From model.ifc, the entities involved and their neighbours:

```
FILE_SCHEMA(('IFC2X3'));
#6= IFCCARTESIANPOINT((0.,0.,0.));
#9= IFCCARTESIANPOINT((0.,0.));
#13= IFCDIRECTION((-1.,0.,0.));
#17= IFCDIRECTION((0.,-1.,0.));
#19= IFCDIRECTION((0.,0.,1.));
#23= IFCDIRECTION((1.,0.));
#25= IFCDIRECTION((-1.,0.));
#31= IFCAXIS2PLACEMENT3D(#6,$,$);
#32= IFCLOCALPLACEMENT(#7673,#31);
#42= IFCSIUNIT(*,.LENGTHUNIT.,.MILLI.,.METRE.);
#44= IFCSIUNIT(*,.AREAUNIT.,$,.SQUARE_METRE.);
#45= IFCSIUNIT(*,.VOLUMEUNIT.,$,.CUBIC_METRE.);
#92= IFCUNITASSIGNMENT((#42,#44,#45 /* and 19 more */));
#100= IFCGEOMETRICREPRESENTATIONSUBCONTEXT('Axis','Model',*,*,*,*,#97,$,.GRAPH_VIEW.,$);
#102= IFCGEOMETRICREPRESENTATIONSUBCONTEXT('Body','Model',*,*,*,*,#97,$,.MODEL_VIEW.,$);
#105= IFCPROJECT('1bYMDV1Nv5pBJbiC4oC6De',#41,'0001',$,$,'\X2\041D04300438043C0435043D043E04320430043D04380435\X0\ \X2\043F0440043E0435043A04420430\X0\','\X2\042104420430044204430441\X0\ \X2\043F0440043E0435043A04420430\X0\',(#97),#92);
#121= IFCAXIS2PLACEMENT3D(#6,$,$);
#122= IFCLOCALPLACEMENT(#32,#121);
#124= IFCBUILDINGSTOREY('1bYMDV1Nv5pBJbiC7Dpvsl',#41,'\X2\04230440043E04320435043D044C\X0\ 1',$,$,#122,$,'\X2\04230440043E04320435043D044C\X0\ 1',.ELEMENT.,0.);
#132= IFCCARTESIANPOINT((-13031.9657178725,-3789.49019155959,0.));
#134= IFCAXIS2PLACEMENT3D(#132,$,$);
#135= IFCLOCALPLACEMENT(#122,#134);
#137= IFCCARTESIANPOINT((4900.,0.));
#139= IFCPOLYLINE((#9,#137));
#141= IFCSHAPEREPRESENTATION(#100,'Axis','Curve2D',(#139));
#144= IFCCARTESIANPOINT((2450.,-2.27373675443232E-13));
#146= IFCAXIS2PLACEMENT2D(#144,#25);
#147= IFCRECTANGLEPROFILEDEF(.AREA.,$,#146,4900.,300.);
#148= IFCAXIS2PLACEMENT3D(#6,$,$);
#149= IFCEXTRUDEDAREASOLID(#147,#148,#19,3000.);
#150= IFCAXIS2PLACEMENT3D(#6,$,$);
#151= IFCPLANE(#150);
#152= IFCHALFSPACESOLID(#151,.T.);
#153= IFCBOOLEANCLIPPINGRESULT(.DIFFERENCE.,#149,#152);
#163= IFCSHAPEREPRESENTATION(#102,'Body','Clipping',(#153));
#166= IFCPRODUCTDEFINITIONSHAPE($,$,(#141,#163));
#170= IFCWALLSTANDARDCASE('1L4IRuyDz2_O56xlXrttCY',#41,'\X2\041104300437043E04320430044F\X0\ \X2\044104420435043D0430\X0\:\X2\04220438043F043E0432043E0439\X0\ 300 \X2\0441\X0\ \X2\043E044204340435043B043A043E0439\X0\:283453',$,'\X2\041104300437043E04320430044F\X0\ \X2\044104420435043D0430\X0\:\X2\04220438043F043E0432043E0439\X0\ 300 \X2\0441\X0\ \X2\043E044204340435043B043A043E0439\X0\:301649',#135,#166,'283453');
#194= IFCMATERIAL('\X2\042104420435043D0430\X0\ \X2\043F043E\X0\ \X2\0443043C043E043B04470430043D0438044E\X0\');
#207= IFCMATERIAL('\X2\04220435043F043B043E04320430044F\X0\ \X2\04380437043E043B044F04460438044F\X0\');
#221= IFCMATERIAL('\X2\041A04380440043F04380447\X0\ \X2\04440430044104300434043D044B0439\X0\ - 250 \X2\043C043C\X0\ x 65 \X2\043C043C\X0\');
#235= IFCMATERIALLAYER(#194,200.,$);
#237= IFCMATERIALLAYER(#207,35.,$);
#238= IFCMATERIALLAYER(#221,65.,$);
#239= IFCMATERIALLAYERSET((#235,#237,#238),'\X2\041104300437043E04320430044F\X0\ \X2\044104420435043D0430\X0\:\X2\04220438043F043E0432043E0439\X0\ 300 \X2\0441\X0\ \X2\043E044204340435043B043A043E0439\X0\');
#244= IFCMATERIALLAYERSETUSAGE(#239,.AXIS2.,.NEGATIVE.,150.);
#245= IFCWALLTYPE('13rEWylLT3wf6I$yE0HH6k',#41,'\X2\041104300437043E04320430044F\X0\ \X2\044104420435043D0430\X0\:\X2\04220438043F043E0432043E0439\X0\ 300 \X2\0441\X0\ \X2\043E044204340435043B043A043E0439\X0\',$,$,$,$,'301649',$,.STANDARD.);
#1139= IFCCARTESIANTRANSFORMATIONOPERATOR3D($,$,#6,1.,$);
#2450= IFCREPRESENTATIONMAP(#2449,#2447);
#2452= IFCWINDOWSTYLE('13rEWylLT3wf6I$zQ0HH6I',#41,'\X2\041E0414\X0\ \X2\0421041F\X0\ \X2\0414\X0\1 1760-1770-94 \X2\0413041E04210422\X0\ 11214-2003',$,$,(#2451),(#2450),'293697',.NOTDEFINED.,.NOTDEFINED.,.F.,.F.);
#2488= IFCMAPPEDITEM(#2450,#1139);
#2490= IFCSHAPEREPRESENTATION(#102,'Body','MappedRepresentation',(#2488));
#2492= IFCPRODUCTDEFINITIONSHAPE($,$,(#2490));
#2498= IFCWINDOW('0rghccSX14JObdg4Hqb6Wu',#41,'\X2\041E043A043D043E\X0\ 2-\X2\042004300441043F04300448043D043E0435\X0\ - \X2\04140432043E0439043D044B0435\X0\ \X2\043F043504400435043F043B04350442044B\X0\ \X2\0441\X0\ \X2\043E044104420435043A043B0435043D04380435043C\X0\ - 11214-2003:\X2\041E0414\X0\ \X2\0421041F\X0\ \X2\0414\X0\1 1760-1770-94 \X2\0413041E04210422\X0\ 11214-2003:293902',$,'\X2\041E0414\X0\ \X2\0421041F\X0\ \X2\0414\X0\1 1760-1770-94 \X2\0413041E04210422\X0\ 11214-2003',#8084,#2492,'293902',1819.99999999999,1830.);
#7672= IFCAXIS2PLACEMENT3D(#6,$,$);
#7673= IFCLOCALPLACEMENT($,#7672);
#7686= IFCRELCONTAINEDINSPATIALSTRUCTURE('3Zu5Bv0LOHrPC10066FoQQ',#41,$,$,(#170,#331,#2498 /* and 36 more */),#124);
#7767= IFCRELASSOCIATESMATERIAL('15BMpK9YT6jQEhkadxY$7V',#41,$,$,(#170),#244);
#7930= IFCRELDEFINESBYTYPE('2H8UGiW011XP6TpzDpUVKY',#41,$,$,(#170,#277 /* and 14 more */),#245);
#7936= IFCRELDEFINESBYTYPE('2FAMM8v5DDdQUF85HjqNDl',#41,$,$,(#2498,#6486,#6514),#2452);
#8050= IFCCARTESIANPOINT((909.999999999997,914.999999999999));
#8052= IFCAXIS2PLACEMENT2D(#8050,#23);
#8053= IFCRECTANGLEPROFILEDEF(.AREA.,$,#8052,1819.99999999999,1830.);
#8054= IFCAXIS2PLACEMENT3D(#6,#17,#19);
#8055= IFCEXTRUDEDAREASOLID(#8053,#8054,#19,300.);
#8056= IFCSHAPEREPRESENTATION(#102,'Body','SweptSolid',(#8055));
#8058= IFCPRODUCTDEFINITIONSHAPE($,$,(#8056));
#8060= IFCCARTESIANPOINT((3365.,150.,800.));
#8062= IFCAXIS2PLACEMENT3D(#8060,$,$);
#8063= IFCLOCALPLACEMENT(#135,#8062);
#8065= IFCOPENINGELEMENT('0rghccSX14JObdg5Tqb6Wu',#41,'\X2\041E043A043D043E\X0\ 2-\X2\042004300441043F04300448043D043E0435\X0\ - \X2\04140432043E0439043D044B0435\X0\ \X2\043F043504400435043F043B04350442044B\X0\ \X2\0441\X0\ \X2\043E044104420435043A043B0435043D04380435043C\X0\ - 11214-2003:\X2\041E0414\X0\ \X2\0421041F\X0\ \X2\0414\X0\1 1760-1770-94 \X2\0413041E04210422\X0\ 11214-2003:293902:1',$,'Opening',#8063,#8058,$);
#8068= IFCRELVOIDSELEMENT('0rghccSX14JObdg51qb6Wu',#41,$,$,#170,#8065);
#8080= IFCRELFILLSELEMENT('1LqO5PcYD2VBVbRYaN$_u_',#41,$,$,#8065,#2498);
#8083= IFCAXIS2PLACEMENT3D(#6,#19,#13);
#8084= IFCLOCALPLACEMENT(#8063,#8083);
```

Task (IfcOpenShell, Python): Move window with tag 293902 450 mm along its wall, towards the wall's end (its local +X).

```python
import ifcopenshell
import ifcopenshell.api.geometry
import ifcopenshell.util.placement

model = ifcopenshell.open("model.ifc")

window = model.by_guid("0rghccSX14JObdg4Hqb6Wu")
opening = window.FillsVoids[0].RelatingOpeningElement
wall = opening.VoidsElements[0].RelatingBuildingElement

wall_matrix = ifcopenshell.util.placement.get_local_placement(wall.ObjectPlacement)
shift = wall_matrix[:3, 0] * 450.0
before = ifcopenshell.util.placement.get_local_placement(window.ObjectPlacement)[:3, 3].copy()

# The window is placed relative to its opening, so it follows when the opening moves.
matrix = ifcopenshell.util.placement.get_local_placement(opening.ObjectPlacement)
matrix[:3, 3] += shift
ifcopenshell.api.geometry.edit_object_placement(
    model, product=opening, matrix=matrix, is_si=False, should_transform_children=True
)

after = ifcopenshell.util.placement.get_local_placement(window.ObjectPlacement)[:3, 3]
print("window moved by", (after - before).round(3) + 0.0)

model.write("model_updated.ifc")
```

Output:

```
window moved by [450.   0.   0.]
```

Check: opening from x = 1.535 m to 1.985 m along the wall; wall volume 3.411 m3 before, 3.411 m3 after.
